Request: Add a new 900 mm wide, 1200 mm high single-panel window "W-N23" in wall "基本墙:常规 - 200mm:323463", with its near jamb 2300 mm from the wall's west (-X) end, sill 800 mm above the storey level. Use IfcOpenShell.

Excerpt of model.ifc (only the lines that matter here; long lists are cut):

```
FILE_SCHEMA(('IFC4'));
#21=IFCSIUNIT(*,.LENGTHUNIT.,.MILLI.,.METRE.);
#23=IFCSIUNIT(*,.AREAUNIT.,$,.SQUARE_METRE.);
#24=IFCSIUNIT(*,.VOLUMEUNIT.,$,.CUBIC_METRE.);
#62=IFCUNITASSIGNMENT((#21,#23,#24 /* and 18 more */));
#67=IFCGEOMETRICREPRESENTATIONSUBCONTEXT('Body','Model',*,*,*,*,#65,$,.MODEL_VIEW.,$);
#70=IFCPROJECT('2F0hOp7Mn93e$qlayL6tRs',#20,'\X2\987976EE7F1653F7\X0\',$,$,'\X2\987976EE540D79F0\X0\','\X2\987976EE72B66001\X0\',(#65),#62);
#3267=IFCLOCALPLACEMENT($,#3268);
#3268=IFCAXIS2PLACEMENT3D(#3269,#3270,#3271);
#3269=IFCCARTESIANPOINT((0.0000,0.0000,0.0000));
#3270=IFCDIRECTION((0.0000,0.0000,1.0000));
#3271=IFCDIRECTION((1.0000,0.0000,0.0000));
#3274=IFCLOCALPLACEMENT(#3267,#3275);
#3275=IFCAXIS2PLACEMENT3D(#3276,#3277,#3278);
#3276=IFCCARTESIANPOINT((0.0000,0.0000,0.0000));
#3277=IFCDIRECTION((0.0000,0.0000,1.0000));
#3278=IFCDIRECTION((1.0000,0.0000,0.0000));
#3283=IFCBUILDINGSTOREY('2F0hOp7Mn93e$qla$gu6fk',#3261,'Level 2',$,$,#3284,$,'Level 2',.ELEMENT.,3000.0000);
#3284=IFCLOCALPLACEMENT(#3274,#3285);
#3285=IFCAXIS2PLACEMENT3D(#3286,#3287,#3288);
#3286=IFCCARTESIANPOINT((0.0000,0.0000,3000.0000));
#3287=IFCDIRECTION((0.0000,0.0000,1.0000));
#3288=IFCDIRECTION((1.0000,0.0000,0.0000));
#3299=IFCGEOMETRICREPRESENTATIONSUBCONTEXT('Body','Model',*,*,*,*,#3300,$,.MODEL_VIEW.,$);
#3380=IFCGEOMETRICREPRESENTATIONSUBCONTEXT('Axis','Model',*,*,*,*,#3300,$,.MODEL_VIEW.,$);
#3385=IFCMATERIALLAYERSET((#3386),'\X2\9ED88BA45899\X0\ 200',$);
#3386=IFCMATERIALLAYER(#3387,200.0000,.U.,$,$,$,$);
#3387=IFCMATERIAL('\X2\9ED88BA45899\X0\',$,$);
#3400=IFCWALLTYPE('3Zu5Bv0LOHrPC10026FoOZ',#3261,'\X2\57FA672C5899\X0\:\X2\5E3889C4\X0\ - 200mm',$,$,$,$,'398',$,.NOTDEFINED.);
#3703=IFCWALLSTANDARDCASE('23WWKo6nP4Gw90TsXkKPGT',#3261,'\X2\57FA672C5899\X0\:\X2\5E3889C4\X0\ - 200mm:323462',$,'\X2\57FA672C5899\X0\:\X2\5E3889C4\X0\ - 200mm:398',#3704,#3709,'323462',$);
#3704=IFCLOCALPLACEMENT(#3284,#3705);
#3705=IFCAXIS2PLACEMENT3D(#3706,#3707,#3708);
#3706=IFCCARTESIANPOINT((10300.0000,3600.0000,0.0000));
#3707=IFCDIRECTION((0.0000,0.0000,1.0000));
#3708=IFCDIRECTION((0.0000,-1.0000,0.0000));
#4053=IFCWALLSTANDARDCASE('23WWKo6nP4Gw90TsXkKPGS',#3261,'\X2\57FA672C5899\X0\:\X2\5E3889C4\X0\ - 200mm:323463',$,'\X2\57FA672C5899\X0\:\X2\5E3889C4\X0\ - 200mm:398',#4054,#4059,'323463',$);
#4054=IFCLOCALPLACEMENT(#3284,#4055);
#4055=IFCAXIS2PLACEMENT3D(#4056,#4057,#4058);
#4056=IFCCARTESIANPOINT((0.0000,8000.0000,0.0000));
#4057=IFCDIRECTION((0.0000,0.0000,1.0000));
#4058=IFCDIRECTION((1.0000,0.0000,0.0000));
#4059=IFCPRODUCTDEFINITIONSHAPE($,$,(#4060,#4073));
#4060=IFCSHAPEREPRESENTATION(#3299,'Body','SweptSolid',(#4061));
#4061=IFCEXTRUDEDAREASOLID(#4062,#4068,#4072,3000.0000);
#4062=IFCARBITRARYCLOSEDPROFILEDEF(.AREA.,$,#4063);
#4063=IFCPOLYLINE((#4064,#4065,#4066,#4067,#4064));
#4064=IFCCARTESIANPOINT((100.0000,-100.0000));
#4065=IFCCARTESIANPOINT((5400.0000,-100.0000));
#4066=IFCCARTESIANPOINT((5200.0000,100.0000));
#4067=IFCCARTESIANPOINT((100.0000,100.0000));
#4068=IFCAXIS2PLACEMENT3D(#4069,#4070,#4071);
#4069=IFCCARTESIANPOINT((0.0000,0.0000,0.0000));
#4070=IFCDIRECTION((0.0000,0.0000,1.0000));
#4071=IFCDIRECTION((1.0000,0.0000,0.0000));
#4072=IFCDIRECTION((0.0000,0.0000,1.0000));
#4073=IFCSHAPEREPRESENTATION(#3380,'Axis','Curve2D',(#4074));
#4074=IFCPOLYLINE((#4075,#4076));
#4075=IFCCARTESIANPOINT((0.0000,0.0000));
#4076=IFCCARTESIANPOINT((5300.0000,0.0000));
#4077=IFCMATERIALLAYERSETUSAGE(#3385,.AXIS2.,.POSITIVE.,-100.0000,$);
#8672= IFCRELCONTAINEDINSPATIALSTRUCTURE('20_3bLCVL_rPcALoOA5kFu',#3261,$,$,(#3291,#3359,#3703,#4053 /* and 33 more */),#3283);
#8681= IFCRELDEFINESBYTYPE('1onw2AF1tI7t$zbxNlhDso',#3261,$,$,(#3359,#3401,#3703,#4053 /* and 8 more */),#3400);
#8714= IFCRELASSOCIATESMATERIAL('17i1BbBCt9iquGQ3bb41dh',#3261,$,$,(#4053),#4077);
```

```python
import numpy as np
import ifcopenshell
import ifcopenshell.api.feature
import ifcopenshell.api.geometry
import ifcopenshell.api.root
import ifcopenshell.api.spatial
import ifcopenshell.geom
import ifcopenshell.util.element
import ifcopenshell.util.placement
import ifcopenshell.util.representation
import ifcopenshell.util.shape
import ifcopenshell.util.unit

model = ifcopenshell.open("model.ifc")
unit_scale = ifcopenshell.util.unit.calculate_unit_scale(model)
settings = ifcopenshell.geom.settings()


def volume(element):
    """Net volume in cubic metres, openings subtracted."""
    shape = ifcopenshell.geom.create_shape(settings, element)
    return ifcopenshell.util.shape.get_volume(shape.geometry)


wall = model.by_id(4053)
storey = ifcopenshell.util.element.get_container(wall, ifc_class="IfcBuildingStorey")
context = ifcopenshell.util.representation.get_context(model, "Model", "Body", "MODEL_VIEW")
before = volume(wall)

width, height, from_end, sill = 0.9, 1.2, 2.3, 0.8  # metres

# The wall runs along its own X axis, and the end named is its -X end.
wall_shape = ifcopenshell.geom.create_shape(settings, wall)
x, y, z = ifcopenshell.util.shape.get_vertices(wall_shape.geometry).T
start = x.min() + from_end
face, thickness = float(y.min()), float(y.max() - y.min())
wall_matrix = ifcopenshell.util.placement.get_local_placement(wall.ObjectPlacement)
level = ifcopenshell.util.placement.get_local_placement(storey.ObjectPlacement)[2, 3]


def in_wall(x, y):
    """Placement at x, y metres in the wall's axes, at sill height."""
    matrix = wall_matrix.copy()
    matrix[:, 3] = wall_matrix @ np.array([x / unit_scale, y / unit_scale, 0.0, 1.0])
    matrix[2, 3] = level + sill / unit_scale
    return matrix


# Opening: a box that overshoots both wall faces by 50 mm.
opening = ifcopenshell.api.root.create_entity(model, ifc_class="IfcOpeningElement", predefined_type="OPENING")
box = ifcopenshell.api.geometry.add_wall_representation(
    model, context=context, length=width, height=height, thickness=thickness + 0.1
)
ifcopenshell.api.geometry.assign_representation(model, product=opening, representation=box)
ifcopenshell.api.geometry.edit_object_placement(model, product=opening, matrix=in_wall(start, face - 0.05), is_si=False)
ifcopenshell.api.feature.add_feature(model, feature=opening, element=wall)

window = ifcopenshell.api.root.create_entity(model, ifc_class="IfcWindow", name="W-N23", predefined_type="WINDOW")
window.OverallWidth, window.OverallHeight = width / unit_scale, height / unit_scale
window.PartitioningType = "SINGLE_PANEL"
body = ifcopenshell.api.geometry.add_window_representation(
    model,
    context=context,
    overall_width=window.OverallWidth,
    overall_height=window.OverallHeight,
    partition_type="SINGLE_PANEL",
)
ifcopenshell.api.geometry.assign_representation(model, product=window, representation=body)
ifcopenshell.api.spatial.assign_container(model, products=[window], relating_structure=storey)
ifcopenshell.api.feature.add_filling(model, opening=opening, element=window)

# Centre the window in the wall's thickness.
ifcopenshell.api.geometry.edit_object_placement(model, product=window, matrix=in_wall(start, face), is_si=False)
window_shape = ifcopenshell.geom.create_shape(settings, window)
depth = ifcopenshell.util.shape.get_vertices(window_shape.geometry)[:, 1]
offset = face + thickness / 2 - (depth.min() + depth.max()) / 2
ifcopenshell.api.geometry.edit_object_placement(model, product=window, matrix=in_wall(start, offset), is_si=False)

after = volume(wall)

print(f"wall volume {before:.3f} -> {after:.3f} m3")

model.write("model_rev.ifc")
```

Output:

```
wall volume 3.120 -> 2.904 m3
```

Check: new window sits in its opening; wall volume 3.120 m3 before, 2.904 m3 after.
